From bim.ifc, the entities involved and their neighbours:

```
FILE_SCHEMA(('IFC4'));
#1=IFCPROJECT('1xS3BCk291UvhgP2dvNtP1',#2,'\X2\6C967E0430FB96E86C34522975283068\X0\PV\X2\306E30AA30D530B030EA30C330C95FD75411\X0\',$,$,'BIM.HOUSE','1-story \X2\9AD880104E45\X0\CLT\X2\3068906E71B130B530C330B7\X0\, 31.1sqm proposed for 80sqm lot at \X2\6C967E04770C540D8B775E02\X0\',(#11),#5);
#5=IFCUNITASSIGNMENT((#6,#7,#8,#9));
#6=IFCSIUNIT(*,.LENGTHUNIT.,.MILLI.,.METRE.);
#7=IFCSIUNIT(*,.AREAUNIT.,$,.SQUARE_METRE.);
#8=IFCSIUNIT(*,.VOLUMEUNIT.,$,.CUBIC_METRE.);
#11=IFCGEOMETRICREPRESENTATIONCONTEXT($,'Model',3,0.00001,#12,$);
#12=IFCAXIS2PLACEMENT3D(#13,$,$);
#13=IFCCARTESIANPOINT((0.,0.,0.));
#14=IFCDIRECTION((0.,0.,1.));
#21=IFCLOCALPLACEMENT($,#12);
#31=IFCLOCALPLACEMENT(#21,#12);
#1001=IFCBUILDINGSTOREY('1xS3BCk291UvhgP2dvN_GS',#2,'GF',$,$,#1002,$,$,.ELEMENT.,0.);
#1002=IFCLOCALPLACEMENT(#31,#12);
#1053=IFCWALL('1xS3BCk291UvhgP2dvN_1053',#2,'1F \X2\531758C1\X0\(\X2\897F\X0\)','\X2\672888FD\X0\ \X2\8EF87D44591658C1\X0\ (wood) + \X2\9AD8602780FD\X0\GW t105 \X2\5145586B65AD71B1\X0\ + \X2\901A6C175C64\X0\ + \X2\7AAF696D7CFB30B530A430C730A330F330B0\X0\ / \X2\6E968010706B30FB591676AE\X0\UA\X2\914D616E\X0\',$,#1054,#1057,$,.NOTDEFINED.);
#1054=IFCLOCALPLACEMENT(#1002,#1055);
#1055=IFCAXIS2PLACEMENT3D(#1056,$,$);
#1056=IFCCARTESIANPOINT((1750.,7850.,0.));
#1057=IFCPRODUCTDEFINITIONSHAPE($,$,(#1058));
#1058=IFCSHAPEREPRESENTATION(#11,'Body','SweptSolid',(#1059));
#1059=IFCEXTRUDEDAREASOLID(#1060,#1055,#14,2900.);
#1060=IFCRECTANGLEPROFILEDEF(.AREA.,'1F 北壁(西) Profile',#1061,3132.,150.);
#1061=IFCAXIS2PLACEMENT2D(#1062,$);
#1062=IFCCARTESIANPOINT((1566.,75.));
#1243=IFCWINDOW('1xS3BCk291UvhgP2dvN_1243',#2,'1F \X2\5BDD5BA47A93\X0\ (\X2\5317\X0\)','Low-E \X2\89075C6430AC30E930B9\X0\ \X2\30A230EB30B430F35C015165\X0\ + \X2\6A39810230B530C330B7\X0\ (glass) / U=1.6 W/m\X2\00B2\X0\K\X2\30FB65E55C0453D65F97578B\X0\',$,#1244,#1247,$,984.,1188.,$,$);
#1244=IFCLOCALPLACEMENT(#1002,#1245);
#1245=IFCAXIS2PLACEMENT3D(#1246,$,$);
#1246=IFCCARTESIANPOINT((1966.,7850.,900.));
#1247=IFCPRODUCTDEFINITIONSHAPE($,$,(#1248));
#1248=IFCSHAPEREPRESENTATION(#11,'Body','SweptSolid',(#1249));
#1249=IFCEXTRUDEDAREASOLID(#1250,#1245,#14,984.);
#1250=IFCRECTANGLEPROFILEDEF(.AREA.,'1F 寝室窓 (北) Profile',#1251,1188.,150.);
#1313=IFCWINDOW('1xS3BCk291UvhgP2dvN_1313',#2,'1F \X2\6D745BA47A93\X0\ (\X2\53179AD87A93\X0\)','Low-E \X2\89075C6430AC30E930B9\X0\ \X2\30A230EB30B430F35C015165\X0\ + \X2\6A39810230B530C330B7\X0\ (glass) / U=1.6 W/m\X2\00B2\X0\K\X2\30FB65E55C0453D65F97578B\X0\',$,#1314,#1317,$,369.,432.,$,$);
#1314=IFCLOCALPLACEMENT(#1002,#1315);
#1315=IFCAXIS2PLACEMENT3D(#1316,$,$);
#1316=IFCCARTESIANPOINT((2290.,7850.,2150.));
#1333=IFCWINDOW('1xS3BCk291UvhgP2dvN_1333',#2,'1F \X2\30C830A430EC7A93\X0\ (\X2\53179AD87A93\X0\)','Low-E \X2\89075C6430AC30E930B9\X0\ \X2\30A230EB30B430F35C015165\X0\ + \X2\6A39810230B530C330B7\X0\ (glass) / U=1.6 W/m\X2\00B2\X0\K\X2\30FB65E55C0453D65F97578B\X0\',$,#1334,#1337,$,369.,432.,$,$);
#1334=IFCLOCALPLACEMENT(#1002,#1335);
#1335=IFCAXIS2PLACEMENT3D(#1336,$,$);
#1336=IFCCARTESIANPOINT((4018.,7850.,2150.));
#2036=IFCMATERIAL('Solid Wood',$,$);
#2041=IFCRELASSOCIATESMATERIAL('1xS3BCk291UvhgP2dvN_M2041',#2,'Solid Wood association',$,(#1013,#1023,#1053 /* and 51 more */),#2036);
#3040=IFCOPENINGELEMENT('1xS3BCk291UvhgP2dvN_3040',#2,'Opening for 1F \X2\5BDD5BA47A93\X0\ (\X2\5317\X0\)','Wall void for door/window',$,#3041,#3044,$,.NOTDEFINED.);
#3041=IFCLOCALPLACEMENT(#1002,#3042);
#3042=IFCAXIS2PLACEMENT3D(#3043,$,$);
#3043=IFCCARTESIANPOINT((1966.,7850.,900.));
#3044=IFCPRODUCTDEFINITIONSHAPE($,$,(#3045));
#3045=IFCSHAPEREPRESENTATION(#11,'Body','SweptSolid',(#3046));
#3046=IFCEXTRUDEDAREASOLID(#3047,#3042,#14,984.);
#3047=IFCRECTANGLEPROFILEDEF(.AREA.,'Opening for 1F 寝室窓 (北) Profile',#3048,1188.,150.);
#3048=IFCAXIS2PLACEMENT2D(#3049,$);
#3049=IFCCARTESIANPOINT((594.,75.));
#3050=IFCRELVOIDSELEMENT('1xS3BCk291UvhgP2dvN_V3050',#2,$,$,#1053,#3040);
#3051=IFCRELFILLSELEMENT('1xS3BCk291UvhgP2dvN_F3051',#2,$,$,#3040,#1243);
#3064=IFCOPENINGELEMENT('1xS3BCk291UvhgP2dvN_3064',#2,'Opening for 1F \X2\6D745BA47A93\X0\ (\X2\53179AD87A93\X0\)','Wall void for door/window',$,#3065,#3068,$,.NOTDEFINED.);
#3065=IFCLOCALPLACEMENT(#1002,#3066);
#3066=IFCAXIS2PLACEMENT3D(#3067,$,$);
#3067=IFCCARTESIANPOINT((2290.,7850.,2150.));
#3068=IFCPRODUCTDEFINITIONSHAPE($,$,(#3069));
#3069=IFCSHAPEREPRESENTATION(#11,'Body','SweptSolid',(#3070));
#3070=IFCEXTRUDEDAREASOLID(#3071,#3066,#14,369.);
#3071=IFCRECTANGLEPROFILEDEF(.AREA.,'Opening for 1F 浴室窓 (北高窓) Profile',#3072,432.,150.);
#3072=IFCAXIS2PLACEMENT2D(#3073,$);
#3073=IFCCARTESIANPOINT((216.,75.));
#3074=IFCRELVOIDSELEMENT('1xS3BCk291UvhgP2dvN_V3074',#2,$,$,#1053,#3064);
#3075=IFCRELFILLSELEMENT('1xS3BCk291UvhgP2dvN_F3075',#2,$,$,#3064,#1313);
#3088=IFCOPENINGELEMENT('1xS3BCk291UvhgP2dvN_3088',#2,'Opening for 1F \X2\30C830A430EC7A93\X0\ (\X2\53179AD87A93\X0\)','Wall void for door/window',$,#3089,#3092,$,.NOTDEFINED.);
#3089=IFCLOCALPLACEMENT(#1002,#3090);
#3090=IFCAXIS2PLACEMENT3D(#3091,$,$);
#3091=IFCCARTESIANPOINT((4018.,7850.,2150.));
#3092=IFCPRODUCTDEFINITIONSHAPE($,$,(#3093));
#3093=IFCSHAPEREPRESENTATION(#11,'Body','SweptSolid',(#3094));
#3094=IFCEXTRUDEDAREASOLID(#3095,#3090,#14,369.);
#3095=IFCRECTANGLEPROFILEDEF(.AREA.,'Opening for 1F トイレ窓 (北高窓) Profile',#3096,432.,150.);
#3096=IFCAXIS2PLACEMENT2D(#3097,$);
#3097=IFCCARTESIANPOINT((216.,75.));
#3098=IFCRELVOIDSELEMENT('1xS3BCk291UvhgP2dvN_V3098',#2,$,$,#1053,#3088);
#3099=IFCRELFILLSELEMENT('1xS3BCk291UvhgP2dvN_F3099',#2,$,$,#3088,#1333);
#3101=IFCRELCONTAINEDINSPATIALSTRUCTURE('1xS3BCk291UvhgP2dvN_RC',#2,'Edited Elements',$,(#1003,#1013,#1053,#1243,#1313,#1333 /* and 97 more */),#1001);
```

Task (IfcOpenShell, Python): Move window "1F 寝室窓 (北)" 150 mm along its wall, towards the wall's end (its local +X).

```python
import ifcopenshell
import ifcopenshell.api.geometry
import ifcopenshell.util.placement
import ifcopenshell.util.unit

model = ifcopenshell.open("bim.ifc")
unit_scale = ifcopenshell.util.unit.calculate_unit_scale(model)

window = model.by_guid("1xS3BCk291UvhgP2dvN_1243")
opening = window.FillsVoids[0].RelatingOpeningElement
wall = opening.VoidsElements[0].RelatingBuildingElement

wall_matrix = ifcopenshell.util.placement.get_local_placement(wall.ObjectPlacement)
shift = wall_matrix[:3, 0] * 0.15 / unit_scale
before = ifcopenshell.util.placement.get_local_placement(window.ObjectPlacement)[:3, 3].copy()

# The window is not placed relative to its opening, so move both.
for product in (opening, window):
    matrix = ifcopenshell.util.placement.get_local_placement(product.ObjectPlacement)
    matrix[:3, 3] += shift
    ifcopenshell.api.geometry.edit_object_placement(model, product=product, matrix=matrix, is_si=False)

after = ifcopenshell.util.placement.get_local_placement(window.ObjectPlacement)[:3, 3]
print("window moved by", (after - before).round(3) + 0.0)

model.write("bim_updated.ifc")
```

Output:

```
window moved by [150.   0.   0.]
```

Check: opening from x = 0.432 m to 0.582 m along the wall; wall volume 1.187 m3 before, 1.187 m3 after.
